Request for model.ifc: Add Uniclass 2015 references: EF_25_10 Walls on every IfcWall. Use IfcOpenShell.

First a look at what the model holds.

```python
import ifcopenshell

model = ifcopenshell.open("model.ifc")
print(model.schema)
print("classifications:", [c.Name for c in model.by_type("IfcClassification")])
for ifc_class in ("IfcDoor", "IfcRoof", "IfcStair", "IfcWall", "IfcWindow"):
    print(ifc_class, len(model.by_type(ifc_class)))
```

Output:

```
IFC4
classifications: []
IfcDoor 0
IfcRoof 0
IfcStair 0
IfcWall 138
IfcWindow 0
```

```python
import ifcopenshell
import ifcopenshell.api.classification

model = ifcopenshell.open("model.ifc")

system = ifcopenshell.api.classification.add_classification(model, classification="Uniclass 2015")

codes = {
    "IfcWall": ("EF_25_10", "Walls"),
}
for ifc_class, (code, name) in codes.items():
    products = model.by_type(ifc_class)
    ifcopenshell.api.classification.add_reference(
        model, products=products, classification=system, identification=code, name=name
    )
    print(code, len(products))

model.write("model_updated.ifc")
```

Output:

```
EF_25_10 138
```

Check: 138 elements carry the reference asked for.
